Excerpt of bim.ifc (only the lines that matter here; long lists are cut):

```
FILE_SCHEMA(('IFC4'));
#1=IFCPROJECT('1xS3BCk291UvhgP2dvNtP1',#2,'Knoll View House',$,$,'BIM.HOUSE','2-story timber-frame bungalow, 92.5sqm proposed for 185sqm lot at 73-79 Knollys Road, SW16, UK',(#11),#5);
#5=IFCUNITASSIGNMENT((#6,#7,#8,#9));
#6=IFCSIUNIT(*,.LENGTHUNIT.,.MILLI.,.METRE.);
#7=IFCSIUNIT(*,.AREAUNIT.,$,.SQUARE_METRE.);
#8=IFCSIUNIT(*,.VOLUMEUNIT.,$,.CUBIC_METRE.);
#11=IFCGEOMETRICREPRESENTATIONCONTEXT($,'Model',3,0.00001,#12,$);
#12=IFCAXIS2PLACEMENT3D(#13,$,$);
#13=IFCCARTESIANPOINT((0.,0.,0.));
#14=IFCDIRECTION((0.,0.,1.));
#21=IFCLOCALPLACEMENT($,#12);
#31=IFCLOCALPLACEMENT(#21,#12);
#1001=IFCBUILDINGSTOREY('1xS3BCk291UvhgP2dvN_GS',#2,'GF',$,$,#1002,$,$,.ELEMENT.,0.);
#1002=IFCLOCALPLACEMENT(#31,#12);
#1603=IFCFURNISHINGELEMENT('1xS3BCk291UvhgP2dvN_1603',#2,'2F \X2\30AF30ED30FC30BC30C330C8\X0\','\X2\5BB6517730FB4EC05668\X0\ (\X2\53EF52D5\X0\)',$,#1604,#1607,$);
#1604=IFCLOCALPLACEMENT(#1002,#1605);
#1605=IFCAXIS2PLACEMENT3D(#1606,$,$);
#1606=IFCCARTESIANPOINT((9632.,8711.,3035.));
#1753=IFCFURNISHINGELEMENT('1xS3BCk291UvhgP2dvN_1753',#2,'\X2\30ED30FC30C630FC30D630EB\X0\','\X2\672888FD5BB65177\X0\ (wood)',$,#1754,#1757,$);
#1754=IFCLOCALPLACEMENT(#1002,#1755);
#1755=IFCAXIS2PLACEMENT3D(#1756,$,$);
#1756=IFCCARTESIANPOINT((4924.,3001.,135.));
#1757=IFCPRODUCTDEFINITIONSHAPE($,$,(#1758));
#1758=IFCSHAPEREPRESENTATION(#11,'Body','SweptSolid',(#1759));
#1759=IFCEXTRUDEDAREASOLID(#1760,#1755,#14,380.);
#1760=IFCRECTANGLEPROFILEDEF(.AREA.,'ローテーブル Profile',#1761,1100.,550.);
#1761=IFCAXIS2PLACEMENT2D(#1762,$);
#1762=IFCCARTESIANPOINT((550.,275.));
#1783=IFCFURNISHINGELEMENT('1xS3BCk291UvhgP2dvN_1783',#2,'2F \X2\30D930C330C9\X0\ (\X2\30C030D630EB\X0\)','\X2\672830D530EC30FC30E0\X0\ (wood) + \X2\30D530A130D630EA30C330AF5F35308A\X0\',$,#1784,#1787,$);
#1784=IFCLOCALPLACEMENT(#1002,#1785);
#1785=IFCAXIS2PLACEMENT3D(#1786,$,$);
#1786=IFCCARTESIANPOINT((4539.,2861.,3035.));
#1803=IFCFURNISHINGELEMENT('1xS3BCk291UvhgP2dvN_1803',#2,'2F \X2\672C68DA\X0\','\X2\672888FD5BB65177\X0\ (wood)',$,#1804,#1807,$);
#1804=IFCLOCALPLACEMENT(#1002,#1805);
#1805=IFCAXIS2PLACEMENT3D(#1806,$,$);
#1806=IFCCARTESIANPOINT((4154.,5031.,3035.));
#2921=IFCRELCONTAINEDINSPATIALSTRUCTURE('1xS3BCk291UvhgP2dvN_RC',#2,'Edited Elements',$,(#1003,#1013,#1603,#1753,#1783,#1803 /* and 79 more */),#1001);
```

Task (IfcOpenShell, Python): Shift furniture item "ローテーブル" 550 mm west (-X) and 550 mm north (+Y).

```python
import ifcopenshell
import ifcopenshell.api.geometry
import ifcopenshell.util.placement

model = ifcopenshell.open("bim.ifc")

item = model.by_guid("1xS3BCk291UvhgP2dvN_1753")
matrix = ifcopenshell.util.placement.get_local_placement(item.ObjectPlacement)
matrix[0, 3] -= 550.0
matrix[1, 3] += 550.0
ifcopenshell.api.geometry.edit_object_placement(model, product=item, matrix=matrix, is_si=False)

print(ifcopenshell.util.placement.get_local_placement(item.ObjectPlacement).round(3) + 0.0)

model.write("bim_rev.ifc")
```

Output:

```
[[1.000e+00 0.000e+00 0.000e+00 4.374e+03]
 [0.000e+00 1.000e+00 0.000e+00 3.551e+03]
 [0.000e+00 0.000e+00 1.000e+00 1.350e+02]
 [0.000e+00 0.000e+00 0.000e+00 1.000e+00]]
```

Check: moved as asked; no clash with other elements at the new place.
